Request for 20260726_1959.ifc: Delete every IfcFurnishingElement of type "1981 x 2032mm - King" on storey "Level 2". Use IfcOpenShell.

First a look at what the model holds.

```python
import ifcopenshell
import ifcopenshell.util.element

model = ifcopenshell.open("20260726_1959.ifc")
print(model.schema)
storey = next(s for s in model.by_type("IfcBuildingStorey") if s.Name == "Level 2")
furniture = [e for e in ifcopenshell.util.element.get_decomposition(storey) if e.is_a("IfcFurnishingElement")]
seen = {}
for e in furniture:
    element_type = ifcopenshell.util.element.get_type(e)
    name = element_type.Name if element_type not in (None, e) else None
    seen[name] = seen.get(name, 0) + 1
for name, count in sorted(seen.items(), key=str):
    print(count, "x", name)
```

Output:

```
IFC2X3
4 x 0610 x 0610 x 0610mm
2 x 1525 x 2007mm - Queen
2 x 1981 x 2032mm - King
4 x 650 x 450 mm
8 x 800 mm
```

```python
import ifcopenshell
import ifcopenshell.api.root
import ifcopenshell.util.element

model = ifcopenshell.open("20260726_1959.ifc")

storey = next(s for s in model.by_type("IfcBuildingStorey") if s.Name == "Level 2")
furniture = [e for e in ifcopenshell.util.element.get_decomposition(storey) if e.is_a("IfcFurnishingElement")]
targets = [e for e in furniture if (t := ifcopenshell.util.element.get_type(e)) not in (None, e) and t.Name == "1981 x 2032mm - King"]

for e in targets:
    ifcopenshell.api.root.remove_product(model, product=e)
print(len(targets), "removed")

model.write("20260726_1959_updated.ifc")
```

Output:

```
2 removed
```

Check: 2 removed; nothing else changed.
